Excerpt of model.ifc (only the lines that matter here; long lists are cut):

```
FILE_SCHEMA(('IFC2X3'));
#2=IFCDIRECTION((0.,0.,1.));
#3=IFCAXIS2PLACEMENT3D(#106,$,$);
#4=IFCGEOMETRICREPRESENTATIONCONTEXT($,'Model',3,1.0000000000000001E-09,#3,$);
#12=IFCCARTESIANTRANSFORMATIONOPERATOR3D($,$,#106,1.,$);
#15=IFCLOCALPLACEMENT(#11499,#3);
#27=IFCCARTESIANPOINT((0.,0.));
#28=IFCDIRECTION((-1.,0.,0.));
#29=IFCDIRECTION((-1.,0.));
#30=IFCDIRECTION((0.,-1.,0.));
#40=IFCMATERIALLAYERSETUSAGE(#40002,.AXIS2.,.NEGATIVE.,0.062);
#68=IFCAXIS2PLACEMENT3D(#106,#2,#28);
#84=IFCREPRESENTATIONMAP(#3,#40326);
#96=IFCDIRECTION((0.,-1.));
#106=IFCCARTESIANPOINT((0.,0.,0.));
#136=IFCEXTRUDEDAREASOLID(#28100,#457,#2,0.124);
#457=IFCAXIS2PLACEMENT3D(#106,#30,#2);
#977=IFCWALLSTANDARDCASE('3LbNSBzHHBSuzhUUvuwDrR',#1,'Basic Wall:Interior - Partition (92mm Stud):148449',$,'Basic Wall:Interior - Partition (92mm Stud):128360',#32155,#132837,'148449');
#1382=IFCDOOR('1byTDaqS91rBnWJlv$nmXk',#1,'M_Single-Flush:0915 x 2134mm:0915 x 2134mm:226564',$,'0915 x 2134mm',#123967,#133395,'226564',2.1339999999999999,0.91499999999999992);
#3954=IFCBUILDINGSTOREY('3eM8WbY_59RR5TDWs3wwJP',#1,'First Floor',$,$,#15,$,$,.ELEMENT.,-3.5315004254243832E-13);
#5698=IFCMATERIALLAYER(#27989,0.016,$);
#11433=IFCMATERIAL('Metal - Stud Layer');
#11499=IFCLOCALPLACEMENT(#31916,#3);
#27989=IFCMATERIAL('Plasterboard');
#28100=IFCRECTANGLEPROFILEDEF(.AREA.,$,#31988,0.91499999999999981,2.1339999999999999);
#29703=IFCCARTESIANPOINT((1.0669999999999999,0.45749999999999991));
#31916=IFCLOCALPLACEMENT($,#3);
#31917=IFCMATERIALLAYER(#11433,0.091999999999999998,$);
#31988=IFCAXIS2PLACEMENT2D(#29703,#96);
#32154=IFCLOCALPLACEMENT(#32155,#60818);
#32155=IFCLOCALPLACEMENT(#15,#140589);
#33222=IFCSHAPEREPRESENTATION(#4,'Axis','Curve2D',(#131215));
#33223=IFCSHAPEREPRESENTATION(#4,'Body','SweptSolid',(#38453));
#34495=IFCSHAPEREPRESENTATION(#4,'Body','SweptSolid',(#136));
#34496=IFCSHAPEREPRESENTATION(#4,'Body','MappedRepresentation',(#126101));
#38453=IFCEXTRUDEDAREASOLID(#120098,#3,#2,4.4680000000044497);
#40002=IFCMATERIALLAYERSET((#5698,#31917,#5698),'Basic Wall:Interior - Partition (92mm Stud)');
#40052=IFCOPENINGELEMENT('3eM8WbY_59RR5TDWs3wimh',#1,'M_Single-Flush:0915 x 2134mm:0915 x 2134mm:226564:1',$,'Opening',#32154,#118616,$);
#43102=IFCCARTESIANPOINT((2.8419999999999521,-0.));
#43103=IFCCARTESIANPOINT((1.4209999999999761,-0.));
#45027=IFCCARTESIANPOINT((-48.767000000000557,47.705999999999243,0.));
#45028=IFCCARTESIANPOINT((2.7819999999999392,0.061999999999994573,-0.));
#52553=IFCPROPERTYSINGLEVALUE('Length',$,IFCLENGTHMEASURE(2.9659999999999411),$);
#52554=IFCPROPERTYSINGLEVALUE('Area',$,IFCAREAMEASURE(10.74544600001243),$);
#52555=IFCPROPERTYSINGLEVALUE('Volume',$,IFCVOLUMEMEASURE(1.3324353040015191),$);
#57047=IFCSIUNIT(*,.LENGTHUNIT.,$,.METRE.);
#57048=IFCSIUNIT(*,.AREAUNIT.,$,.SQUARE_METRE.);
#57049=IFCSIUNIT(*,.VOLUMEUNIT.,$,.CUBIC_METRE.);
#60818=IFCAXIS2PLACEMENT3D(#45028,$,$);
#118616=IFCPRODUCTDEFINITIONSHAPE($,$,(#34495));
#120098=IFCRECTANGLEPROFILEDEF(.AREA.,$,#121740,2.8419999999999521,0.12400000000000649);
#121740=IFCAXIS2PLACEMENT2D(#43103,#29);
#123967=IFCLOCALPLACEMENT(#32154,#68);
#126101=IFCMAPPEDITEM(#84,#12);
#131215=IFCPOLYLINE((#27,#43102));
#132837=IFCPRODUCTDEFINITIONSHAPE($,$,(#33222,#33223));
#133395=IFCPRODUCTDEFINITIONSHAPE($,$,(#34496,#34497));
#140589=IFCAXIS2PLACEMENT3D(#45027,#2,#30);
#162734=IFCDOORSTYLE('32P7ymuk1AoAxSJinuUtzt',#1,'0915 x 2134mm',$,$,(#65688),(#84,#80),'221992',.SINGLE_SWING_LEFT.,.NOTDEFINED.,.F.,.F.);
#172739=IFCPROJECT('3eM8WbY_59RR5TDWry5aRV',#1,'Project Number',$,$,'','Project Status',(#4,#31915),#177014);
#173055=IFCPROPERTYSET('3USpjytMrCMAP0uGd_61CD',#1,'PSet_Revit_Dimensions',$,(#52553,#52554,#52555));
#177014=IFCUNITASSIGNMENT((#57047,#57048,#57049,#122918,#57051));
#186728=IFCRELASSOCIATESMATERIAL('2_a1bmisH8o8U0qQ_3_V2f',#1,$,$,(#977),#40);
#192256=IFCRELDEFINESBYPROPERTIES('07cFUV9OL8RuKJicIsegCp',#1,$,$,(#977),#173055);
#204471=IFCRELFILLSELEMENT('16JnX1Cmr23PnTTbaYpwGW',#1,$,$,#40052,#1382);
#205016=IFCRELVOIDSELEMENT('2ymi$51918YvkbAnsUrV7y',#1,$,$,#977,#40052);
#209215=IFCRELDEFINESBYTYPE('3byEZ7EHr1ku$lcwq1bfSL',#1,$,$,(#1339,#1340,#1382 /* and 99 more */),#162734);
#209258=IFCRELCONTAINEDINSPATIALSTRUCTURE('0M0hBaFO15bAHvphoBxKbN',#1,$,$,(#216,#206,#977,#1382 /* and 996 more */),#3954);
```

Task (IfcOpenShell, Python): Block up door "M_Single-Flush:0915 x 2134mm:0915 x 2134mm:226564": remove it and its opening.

```python
import ifcopenshell
import ifcopenshell.api.feature
import ifcopenshell.api.pset
import ifcopenshell.api.root
import ifcopenshell.geom
import ifcopenshell.util.element
import ifcopenshell.util.shape
import ifcopenshell.util.unit

model = ifcopenshell.open("model.ifc")
area_scale = ifcopenshell.util.unit.calculate_unit_scale(model, "AREAUNIT")
volume_scale = ifcopenshell.util.unit.calculate_unit_scale(model, "VOLUMEUNIT")
settings = ifcopenshell.geom.settings()


def volume(element):
    """Net volume in cubic metres, openings subtracted."""
    shape = ifcopenshell.geom.create_shape(settings, element)
    return ifcopenshell.util.shape.get_volume(shape.geometry)


door = model.by_guid("1byTDaqS91rBnWJlv$nmXk")
opening = door.FillsVoids[0].RelatingOpeningElement
wall = opening.VoidsElements[0].RelatingBuildingElement
before = volume(wall)

ifcopenshell.api.root.remove_product(model, product=door)
ifcopenshell.api.feature.remove_feature(model, feature=opening)

after = volume(wall)
thickness = 0.124  # wall thickness in metres

# Update the wall's stored quantities.
pset = model.by_id(ifcopenshell.util.element.get_pset(wall, "PSet_Revit_Dimensions", should_inherit=False)["id"])
ifcopenshell.api.pset.edit_pset(model, pset=pset, properties={
    "Area": model.create_entity("IfcAreaMeasure", after / thickness / area_scale),
    "Volume": model.create_entity("IfcVolumeMeasure", after / volume_scale),
})

print(f"wall volume {before:.3f} -> {after:.3f} m3")

model.write("model_updated.ifc")
```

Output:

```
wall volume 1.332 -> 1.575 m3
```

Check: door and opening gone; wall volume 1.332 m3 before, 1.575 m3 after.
